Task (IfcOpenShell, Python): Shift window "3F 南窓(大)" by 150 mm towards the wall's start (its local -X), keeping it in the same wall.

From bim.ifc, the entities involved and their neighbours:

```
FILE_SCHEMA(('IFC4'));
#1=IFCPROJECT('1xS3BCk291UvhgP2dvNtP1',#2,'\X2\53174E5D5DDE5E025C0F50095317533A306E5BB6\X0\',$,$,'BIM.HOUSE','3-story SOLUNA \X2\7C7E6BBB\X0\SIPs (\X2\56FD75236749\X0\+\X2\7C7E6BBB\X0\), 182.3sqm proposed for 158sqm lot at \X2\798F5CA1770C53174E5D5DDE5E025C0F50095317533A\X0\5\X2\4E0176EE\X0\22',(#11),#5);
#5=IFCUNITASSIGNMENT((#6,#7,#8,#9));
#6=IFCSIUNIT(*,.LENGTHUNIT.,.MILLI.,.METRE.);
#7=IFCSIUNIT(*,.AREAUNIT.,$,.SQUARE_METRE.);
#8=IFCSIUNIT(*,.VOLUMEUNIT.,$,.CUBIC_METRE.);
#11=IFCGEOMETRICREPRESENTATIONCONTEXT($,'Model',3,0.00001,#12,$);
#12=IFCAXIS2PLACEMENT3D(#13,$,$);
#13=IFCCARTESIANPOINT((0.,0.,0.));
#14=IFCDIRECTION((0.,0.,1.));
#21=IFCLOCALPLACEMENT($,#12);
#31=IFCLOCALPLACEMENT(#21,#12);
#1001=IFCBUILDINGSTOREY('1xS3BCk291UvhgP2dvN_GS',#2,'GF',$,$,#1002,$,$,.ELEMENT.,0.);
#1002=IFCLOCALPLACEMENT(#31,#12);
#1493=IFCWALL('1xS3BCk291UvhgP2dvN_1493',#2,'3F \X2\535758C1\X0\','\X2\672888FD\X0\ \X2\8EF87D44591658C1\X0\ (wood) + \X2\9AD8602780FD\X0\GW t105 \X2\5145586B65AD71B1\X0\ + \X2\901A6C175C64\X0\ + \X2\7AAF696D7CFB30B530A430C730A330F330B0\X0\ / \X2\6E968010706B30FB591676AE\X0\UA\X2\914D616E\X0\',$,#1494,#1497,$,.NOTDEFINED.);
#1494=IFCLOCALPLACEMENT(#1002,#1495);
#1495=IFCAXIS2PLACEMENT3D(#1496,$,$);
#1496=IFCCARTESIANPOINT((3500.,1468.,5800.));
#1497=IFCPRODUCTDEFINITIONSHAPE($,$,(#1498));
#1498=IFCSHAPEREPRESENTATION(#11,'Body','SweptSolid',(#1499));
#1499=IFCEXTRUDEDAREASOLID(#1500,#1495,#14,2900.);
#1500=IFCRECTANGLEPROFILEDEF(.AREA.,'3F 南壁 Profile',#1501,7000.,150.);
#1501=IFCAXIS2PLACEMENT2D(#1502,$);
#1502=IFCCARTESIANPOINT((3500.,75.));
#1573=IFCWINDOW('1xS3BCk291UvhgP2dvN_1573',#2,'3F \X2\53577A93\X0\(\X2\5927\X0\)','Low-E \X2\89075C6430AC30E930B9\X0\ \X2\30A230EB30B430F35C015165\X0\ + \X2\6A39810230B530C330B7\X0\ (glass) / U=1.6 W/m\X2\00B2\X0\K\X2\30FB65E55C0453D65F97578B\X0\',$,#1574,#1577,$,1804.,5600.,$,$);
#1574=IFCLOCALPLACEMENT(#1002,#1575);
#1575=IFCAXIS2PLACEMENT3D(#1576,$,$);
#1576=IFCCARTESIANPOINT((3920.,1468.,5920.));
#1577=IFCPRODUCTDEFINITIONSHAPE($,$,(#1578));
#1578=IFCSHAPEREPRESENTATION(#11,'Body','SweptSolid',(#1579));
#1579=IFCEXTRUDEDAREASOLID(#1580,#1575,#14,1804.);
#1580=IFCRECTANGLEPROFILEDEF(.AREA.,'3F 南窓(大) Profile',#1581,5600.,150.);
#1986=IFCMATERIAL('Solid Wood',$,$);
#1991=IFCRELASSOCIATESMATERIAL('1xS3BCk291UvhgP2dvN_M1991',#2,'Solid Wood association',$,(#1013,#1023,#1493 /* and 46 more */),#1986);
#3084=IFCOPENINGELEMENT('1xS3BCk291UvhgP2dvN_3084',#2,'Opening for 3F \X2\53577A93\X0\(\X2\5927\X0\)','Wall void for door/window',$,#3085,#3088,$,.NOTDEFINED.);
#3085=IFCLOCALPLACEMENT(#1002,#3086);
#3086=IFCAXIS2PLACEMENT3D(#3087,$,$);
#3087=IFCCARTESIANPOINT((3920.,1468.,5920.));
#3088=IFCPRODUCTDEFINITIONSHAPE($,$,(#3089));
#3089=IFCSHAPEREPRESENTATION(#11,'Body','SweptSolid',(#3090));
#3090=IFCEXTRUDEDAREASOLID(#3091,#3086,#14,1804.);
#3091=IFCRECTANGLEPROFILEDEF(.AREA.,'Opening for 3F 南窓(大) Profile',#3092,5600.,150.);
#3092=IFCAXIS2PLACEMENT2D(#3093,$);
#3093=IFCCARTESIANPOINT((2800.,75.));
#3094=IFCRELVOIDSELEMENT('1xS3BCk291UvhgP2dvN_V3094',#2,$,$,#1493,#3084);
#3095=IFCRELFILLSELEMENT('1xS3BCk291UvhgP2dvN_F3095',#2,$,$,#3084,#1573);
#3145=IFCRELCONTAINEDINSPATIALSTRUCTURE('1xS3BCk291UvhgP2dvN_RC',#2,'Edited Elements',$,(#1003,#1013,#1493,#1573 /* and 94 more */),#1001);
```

```python
import ifcopenshell
import ifcopenshell.api.geometry
import ifcopenshell.util.placement

model = ifcopenshell.open("bim.ifc")

window = model.by_guid("1xS3BCk291UvhgP2dvN_1573")
opening = window.FillsVoids[0].RelatingOpeningElement
wall = opening.VoidsElements[0].RelatingBuildingElement

wall_matrix = ifcopenshell.util.placement.get_local_placement(wall.ObjectPlacement)
shift = wall_matrix[:3, 0] * -150.0
before = ifcopenshell.util.placement.get_local_placement(window.ObjectPlacement)[:3, 3].copy()

# The window is not placed relative to its opening, so move both.
for product in (opening, window):
    matrix = ifcopenshell.util.placement.get_local_placement(product.ObjectPlacement)
    matrix[:3, 3] += shift
    ifcopenshell.api.geometry.edit_object_placement(model, product=product, matrix=matrix, is_si=False)

after = ifcopenshell.util.placement.get_local_placement(window.ObjectPlacement)[:3, 3]
print("window moved by", (after - before).round(3) + 0.0)

model.write("bim_rev.ifc")
```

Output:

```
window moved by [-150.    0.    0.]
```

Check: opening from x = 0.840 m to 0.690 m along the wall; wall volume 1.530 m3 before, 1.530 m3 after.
